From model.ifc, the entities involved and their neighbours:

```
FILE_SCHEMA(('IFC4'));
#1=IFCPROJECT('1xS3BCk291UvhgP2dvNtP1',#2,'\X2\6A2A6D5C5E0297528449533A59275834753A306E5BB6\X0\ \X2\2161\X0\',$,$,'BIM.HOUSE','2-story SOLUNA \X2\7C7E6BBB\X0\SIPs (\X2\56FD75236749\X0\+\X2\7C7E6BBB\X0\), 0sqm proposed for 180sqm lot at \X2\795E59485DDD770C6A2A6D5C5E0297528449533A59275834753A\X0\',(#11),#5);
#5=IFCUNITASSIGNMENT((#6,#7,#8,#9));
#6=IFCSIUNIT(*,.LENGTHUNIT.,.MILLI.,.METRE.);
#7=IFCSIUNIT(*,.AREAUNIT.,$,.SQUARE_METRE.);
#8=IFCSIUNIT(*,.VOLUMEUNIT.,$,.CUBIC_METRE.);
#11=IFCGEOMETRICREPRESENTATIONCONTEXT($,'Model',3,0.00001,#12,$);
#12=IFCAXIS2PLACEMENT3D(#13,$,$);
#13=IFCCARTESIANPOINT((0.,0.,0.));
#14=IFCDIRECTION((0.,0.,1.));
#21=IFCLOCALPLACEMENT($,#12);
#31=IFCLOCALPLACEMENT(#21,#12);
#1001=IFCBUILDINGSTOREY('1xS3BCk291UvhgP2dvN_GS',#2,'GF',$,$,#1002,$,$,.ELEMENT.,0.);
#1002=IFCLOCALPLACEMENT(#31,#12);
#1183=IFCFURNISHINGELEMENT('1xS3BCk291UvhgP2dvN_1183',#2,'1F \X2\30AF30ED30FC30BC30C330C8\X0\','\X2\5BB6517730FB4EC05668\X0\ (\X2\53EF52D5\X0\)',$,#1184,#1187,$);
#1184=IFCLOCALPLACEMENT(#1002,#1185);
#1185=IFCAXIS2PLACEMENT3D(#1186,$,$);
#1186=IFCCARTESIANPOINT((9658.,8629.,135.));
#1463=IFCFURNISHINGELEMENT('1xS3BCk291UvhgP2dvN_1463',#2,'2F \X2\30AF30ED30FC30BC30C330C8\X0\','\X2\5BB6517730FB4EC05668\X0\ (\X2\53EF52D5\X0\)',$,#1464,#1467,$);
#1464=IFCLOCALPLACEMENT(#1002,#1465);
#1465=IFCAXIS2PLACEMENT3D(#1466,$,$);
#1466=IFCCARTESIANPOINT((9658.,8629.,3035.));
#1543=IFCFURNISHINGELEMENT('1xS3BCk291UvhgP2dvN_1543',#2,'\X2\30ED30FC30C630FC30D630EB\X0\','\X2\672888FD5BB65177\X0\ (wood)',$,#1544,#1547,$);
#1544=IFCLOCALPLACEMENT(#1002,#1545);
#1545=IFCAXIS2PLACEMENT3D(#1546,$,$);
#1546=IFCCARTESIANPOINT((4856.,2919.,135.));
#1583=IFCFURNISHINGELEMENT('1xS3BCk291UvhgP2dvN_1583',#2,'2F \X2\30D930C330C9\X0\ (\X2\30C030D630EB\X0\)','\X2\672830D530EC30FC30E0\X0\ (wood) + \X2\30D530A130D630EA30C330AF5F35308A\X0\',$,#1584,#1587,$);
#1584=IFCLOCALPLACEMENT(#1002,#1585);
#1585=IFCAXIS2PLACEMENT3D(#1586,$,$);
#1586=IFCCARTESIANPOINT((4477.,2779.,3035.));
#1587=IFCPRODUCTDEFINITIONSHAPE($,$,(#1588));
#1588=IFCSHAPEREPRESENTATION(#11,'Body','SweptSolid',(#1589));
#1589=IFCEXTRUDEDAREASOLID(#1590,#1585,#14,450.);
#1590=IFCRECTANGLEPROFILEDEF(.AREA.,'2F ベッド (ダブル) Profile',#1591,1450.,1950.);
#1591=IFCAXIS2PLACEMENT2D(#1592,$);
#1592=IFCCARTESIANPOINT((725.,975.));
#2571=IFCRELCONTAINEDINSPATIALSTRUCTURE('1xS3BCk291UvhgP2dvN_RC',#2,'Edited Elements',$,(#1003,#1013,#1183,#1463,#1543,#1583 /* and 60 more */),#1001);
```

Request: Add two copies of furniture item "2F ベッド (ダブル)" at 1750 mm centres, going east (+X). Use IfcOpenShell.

```python
import numpy as np
import ifcopenshell
import ifcopenshell.api.geometry
import ifcopenshell.api.root
import ifcopenshell.util.element
import ifcopenshell.util.placement

model = ifcopenshell.open("model.ifc")


def reuse_history(source, copy):
    """copy_class also copies each property set's owner history, people and application; keep the originals."""
    for rel in copy.IsDefinedBy:
        if rel.is_a("IfcRelDefinesByProperties") and (history := rel.RelatingPropertyDefinition.OwnerHistory):
            rel.RelatingPropertyDefinition.OwnerHistory = source.OwnerHistory
            ifcopenshell.util.element.remove_deep2(model, history)


source = model.by_guid("1xS3BCk291UvhgP2dvN_1583")
base = ifcopenshell.util.placement.get_local_placement(source.ObjectPlacement)
step = np.array([1.0, 0.0, 0.0]) * 1750.0

for i in range(1, 3):
    copy = ifcopenshell.api.root.copy_class(model, product=source)
    copy.Representation = ifcopenshell.util.element.copy_deep(
        model, source.Representation, exclude=["IfcGeometricRepresentationContext", "IfcRepresentationMap"]
    )
    reuse_history(source, copy)
    matrix = base.copy()
    matrix[:3, 3] += i * step
    print("added at", matrix[:3, 3].round(3) + 0.0)
    ifcopenshell.api.geometry.edit_object_placement(model, product=copy, matrix=matrix, is_si=False)

model.write("model_rev.ifc")
```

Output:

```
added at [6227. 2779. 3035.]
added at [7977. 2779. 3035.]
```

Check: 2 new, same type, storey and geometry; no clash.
